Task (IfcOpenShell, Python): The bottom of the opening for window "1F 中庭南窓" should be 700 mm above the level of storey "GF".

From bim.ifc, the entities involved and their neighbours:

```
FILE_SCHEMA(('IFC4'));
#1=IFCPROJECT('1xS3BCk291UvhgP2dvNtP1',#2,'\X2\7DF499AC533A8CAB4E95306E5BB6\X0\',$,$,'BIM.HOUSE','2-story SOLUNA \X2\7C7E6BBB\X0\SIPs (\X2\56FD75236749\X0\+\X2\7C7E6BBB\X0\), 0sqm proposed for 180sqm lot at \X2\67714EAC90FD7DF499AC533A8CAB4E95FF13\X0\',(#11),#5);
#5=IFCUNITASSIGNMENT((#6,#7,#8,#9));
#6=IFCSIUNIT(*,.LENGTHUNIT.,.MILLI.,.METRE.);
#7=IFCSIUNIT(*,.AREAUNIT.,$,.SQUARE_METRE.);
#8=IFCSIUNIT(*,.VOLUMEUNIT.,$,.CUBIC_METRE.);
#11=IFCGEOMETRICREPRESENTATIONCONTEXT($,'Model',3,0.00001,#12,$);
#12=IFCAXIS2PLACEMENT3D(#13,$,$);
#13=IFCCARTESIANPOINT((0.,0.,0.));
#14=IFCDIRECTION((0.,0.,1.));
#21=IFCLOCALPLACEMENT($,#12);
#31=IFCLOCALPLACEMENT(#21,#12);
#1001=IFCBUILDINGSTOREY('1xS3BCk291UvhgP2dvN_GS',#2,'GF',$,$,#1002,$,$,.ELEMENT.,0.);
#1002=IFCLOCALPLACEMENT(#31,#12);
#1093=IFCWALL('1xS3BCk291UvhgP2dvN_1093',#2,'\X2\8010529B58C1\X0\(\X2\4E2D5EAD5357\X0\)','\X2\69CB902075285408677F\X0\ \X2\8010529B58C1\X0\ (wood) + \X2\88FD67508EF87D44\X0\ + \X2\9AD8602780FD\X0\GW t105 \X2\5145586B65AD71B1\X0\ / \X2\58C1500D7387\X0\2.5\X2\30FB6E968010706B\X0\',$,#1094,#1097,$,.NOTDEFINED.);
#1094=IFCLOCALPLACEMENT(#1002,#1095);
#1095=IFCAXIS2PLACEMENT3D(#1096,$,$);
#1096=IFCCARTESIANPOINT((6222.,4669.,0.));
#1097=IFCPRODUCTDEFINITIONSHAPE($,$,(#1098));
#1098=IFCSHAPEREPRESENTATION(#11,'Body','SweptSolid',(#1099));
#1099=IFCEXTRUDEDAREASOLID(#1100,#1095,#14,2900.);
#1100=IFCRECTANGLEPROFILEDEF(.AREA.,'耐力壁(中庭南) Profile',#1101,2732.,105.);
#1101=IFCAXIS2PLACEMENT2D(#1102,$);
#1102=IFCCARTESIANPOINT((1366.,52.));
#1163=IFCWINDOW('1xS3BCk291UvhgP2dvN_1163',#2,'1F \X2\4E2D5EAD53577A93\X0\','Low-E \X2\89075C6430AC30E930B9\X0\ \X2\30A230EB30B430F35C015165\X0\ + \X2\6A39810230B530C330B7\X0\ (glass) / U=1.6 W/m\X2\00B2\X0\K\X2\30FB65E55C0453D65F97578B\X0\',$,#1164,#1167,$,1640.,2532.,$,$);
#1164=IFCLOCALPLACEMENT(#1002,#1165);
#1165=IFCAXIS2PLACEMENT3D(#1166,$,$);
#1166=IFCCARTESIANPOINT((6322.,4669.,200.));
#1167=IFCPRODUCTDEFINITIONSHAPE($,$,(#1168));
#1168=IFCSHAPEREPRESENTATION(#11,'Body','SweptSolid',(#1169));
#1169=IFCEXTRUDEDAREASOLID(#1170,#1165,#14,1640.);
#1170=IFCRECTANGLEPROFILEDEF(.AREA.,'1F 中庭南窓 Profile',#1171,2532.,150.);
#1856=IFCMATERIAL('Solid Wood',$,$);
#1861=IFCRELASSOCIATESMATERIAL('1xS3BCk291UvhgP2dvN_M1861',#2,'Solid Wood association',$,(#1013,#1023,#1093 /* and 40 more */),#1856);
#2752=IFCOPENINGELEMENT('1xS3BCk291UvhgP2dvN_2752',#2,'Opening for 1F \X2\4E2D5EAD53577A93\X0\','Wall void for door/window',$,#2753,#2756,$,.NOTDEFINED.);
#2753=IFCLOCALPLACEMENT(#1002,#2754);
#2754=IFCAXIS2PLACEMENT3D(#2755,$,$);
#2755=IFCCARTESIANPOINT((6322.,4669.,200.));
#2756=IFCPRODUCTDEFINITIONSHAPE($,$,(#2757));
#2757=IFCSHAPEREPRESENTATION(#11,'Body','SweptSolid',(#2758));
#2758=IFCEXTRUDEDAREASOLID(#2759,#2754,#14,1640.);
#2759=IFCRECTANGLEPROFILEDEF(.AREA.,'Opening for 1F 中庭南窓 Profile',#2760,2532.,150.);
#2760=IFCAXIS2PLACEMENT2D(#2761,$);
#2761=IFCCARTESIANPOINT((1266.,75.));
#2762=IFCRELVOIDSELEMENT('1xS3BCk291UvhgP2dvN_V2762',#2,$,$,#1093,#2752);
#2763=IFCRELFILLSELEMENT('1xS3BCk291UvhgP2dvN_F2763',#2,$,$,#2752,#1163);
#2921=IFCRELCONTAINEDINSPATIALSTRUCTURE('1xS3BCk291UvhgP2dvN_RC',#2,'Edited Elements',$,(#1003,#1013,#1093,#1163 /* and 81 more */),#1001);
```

```python
import numpy as np
import ifcopenshell
import ifcopenshell.api.geometry
import ifcopenshell.geom
import ifcopenshell.util.element
import ifcopenshell.util.placement
import ifcopenshell.util.shape
import ifcopenshell.util.unit

model = ifcopenshell.open("bim.ifc")
unit_scale = ifcopenshell.util.unit.calculate_unit_scale(model)

window = model.by_guid("1xS3BCk291UvhgP2dvN_1163")
opening = window.FillsVoids[0].RelatingOpeningElement
storey = ifcopenshell.util.element.get_container(window, ifc_class="IfcBuildingStorey")
level = ifcopenshell.util.placement.get_local_placement(storey.ObjectPlacement)[2, 3]

# The opening's origin need not be at the sill, so measure its lowest point.
shape = ifcopenshell.geom.create_shape(ifcopenshell.geom.settings(), opening)
bottom = ifcopenshell.util.shape.get_shape_bottom_elevation(shape, shape.geometry) / unit_scale
dz = level + 700.0 - bottom

shift = np.array([0.0, 0.0, dz])
# The window is not placed relative to its opening, so move both.
for product in (opening, window):
    matrix = ifcopenshell.util.placement.get_local_placement(product.ObjectPlacement)
    matrix[:3, 3] += shift
    ifcopenshell.api.geometry.edit_object_placement(model, product=product, matrix=matrix, is_si=False)

print(f"moved by {dz * unit_scale:+.3f} m")

model.write("bim_rev.ifc")
```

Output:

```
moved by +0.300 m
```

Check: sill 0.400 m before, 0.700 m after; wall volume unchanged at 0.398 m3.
